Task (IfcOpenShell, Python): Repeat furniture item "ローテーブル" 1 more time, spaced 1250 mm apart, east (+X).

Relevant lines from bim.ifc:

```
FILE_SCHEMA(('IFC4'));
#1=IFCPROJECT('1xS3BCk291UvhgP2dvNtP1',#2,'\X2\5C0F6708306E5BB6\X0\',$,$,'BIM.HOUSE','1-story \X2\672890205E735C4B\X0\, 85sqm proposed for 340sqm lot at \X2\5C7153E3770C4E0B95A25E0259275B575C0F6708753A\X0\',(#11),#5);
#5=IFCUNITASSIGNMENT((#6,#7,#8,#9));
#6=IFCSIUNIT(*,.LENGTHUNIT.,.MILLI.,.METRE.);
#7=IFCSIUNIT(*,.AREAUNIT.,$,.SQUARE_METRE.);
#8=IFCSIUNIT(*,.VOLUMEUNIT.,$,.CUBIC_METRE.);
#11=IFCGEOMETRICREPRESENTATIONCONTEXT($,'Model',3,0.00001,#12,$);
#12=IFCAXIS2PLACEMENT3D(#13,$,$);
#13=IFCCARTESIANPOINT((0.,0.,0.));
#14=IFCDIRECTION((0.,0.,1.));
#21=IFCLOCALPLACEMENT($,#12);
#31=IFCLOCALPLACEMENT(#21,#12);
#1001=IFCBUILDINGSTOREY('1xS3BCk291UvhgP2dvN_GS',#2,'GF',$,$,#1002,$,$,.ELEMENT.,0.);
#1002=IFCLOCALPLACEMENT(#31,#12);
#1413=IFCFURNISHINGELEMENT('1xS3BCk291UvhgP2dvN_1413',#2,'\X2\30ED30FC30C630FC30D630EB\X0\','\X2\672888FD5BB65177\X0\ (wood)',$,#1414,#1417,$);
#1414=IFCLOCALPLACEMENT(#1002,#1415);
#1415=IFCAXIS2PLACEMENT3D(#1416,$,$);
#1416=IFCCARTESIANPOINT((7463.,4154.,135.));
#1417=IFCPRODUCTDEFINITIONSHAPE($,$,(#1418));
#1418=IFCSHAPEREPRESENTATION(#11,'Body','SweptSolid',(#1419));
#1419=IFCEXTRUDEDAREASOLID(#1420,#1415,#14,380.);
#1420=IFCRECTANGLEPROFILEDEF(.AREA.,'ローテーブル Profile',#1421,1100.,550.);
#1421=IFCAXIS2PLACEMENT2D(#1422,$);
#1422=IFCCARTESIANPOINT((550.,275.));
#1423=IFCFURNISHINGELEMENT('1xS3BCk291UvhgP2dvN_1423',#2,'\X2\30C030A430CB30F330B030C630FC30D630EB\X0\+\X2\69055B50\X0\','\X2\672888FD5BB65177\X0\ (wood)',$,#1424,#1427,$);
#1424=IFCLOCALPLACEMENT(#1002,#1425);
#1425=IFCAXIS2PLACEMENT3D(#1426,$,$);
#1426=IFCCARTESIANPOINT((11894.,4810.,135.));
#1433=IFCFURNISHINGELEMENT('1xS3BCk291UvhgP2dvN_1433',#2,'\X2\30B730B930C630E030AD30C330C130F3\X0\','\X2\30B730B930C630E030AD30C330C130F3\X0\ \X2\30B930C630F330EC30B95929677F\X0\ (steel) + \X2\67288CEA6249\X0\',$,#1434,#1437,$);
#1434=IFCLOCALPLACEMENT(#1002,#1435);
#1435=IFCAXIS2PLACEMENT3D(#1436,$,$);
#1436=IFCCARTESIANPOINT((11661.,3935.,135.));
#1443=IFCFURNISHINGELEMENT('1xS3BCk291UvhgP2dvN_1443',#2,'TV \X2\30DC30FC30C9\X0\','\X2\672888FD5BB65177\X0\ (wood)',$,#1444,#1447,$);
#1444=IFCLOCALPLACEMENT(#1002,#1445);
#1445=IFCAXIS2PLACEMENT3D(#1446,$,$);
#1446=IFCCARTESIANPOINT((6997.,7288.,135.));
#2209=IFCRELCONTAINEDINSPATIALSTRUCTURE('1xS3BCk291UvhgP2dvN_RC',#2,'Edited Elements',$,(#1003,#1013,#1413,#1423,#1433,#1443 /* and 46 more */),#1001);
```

```python
import numpy as np
import ifcopenshell
import ifcopenshell.api.geometry
import ifcopenshell.api.root
import ifcopenshell.util.element
import ifcopenshell.util.placement
import ifcopenshell.util.unit

model = ifcopenshell.open("bim.ifc")
unit_scale = ifcopenshell.util.unit.calculate_unit_scale(model)


def reuse_history(source, copy):
    """copy_class also copies each property set's owner history, people and application; keep the originals."""
    for rel in copy.IsDefinedBy:
        if rel.is_a("IfcRelDefinesByProperties") and (history := rel.RelatingPropertyDefinition.OwnerHistory):
            rel.RelatingPropertyDefinition.OwnerHistory = source.OwnerHistory
            ifcopenshell.util.element.remove_deep2(model, history)


source = model.by_id(1413)
base = ifcopenshell.util.placement.get_local_placement(source.ObjectPlacement)
step = np.array([1.0, 0.0, 0.0]) * 1.25 / unit_scale

for i in range(1, 2):
    copy = ifcopenshell.api.root.copy_class(model, product=source)
    copy.Representation = ifcopenshell.util.element.copy_deep(
        model, source.Representation, exclude=["IfcGeometricRepresentationContext", "IfcRepresentationMap"]
    )
    reuse_history(source, copy)
    matrix = base.copy()
    matrix[:3, 3] += i * step
    print("added at", matrix[:3, 3].round(3) + 0.0)
    ifcopenshell.api.geometry.edit_object_placement(model, product=copy, matrix=matrix, is_si=False)

model.write("bim-out.ifc")
```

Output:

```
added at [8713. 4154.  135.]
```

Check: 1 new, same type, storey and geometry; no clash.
